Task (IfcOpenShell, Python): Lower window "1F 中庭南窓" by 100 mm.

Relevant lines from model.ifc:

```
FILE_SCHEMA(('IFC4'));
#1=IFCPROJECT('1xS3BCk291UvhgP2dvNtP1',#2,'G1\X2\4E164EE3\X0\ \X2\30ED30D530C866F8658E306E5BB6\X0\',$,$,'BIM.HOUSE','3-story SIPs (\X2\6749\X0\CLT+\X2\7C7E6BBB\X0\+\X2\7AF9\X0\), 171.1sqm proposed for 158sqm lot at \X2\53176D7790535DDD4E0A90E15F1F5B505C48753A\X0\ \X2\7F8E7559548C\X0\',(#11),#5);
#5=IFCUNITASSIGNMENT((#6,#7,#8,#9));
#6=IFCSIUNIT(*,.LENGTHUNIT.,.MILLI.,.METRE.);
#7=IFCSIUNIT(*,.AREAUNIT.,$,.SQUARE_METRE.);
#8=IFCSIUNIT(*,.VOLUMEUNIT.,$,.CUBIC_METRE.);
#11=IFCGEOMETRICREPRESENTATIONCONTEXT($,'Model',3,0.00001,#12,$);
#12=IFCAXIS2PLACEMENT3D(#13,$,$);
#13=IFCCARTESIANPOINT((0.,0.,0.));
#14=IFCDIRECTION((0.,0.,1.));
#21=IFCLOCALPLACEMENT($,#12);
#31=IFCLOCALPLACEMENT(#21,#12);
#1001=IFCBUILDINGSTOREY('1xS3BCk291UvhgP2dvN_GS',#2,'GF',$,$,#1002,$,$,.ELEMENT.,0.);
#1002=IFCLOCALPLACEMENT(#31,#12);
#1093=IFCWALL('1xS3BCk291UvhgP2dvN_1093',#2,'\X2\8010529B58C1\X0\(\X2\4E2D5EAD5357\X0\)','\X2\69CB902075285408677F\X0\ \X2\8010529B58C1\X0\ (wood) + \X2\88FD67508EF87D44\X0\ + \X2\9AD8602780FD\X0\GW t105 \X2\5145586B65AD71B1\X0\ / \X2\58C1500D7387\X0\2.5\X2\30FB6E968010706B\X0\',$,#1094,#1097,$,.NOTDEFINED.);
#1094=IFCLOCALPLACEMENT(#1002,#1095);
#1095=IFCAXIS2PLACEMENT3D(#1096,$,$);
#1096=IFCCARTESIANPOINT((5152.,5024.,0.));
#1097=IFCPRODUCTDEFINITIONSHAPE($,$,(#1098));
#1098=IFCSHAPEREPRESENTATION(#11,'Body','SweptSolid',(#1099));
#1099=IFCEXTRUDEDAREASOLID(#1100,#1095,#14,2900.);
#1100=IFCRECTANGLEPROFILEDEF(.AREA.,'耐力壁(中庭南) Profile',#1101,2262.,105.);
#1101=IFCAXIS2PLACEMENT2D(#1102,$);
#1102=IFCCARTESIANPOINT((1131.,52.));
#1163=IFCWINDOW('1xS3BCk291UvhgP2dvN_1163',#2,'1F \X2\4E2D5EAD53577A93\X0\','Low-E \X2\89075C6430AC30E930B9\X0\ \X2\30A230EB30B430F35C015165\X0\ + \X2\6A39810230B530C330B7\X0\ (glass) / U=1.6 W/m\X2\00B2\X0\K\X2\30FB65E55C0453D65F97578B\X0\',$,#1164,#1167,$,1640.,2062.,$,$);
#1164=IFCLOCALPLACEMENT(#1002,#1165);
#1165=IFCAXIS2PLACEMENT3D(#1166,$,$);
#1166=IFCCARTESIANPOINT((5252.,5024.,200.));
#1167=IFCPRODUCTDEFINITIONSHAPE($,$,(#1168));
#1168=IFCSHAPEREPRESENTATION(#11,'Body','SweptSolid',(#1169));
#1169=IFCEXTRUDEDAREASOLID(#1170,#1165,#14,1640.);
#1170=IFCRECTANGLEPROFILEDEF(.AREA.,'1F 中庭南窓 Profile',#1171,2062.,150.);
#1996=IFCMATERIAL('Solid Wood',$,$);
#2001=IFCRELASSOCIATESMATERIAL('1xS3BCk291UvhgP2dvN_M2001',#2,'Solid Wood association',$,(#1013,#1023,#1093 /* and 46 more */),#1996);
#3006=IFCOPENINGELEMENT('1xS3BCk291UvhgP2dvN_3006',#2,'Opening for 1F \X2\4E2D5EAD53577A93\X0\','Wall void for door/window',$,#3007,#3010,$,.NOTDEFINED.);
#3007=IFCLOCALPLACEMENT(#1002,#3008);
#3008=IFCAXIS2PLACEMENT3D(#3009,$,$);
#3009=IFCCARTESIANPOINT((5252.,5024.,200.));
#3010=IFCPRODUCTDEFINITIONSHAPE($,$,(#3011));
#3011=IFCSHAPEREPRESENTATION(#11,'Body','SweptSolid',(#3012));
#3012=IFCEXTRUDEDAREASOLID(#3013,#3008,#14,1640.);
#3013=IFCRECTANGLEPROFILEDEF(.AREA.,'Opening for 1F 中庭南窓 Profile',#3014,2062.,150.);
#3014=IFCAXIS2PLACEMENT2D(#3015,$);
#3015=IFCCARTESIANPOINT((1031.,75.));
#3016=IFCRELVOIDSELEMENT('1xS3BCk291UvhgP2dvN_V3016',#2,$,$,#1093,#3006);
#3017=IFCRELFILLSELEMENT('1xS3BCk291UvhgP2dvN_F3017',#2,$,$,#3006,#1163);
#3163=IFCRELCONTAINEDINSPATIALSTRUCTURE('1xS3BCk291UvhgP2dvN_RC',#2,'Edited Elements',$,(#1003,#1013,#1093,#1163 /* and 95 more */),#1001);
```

```python
import numpy as np
import ifcopenshell
import ifcopenshell.api.geometry
import ifcopenshell.util.placement
import ifcopenshell.util.unit

model = ifcopenshell.open("model.ifc")
unit_scale = ifcopenshell.util.unit.calculate_unit_scale(model)

window = model.by_guid("1xS3BCk291UvhgP2dvN_1163")
opening = window.FillsVoids[0].RelatingOpeningElement
dz = -0.1 / unit_scale

shift = np.array([0.0, 0.0, dz])
# The window is not placed relative to its opening, so move both.
for product in (opening, window):
    matrix = ifcopenshell.util.placement.get_local_placement(product.ObjectPlacement)
    matrix[:3, 3] += shift
    ifcopenshell.api.geometry.edit_object_placement(model, product=product, matrix=matrix, is_si=False)

print(f"moved by {dz * unit_scale:+.3f} m")

model.write("model_edited.ifc")
```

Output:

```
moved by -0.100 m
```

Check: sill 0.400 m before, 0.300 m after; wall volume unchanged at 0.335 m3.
